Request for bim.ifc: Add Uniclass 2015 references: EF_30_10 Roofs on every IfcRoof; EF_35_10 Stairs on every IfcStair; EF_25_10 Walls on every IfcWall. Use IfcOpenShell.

First a look at what the model holds.

```python
import ifcopenshell

model = ifcopenshell.open("bim.ifc")
print(model.schema)
print("classifications:", [c.Name for c in model.by_type("IfcClassification")])
for ifc_class in ("IfcDoor", "IfcRoof", "IfcStair", "IfcWall", "IfcWindow"):
    print(ifc_class, len(model.by_type(ifc_class)))
```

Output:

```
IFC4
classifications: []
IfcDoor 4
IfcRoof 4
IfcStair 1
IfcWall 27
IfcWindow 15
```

```python
import ifcopenshell
import ifcopenshell.api.classification

model = ifcopenshell.open("bim.ifc")

system = ifcopenshell.api.classification.add_classification(model, classification="Uniclass 2015")

codes = {
    "IfcRoof": ("EF_30_10", "Roofs"),
    "IfcStair": ("EF_35_10", "Stairs"),
    "IfcWall": ("EF_25_10", "Walls"),
}
for ifc_class, (code, name) in codes.items():
    products = model.by_type(ifc_class)
    ifcopenshell.api.classification.add_reference(
        model, products=products, classification=system, identification=code, name=name
    )
    print(code, len(products))

model.write("bim_v2.ifc")
```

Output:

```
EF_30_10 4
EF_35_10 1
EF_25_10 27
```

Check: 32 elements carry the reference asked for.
